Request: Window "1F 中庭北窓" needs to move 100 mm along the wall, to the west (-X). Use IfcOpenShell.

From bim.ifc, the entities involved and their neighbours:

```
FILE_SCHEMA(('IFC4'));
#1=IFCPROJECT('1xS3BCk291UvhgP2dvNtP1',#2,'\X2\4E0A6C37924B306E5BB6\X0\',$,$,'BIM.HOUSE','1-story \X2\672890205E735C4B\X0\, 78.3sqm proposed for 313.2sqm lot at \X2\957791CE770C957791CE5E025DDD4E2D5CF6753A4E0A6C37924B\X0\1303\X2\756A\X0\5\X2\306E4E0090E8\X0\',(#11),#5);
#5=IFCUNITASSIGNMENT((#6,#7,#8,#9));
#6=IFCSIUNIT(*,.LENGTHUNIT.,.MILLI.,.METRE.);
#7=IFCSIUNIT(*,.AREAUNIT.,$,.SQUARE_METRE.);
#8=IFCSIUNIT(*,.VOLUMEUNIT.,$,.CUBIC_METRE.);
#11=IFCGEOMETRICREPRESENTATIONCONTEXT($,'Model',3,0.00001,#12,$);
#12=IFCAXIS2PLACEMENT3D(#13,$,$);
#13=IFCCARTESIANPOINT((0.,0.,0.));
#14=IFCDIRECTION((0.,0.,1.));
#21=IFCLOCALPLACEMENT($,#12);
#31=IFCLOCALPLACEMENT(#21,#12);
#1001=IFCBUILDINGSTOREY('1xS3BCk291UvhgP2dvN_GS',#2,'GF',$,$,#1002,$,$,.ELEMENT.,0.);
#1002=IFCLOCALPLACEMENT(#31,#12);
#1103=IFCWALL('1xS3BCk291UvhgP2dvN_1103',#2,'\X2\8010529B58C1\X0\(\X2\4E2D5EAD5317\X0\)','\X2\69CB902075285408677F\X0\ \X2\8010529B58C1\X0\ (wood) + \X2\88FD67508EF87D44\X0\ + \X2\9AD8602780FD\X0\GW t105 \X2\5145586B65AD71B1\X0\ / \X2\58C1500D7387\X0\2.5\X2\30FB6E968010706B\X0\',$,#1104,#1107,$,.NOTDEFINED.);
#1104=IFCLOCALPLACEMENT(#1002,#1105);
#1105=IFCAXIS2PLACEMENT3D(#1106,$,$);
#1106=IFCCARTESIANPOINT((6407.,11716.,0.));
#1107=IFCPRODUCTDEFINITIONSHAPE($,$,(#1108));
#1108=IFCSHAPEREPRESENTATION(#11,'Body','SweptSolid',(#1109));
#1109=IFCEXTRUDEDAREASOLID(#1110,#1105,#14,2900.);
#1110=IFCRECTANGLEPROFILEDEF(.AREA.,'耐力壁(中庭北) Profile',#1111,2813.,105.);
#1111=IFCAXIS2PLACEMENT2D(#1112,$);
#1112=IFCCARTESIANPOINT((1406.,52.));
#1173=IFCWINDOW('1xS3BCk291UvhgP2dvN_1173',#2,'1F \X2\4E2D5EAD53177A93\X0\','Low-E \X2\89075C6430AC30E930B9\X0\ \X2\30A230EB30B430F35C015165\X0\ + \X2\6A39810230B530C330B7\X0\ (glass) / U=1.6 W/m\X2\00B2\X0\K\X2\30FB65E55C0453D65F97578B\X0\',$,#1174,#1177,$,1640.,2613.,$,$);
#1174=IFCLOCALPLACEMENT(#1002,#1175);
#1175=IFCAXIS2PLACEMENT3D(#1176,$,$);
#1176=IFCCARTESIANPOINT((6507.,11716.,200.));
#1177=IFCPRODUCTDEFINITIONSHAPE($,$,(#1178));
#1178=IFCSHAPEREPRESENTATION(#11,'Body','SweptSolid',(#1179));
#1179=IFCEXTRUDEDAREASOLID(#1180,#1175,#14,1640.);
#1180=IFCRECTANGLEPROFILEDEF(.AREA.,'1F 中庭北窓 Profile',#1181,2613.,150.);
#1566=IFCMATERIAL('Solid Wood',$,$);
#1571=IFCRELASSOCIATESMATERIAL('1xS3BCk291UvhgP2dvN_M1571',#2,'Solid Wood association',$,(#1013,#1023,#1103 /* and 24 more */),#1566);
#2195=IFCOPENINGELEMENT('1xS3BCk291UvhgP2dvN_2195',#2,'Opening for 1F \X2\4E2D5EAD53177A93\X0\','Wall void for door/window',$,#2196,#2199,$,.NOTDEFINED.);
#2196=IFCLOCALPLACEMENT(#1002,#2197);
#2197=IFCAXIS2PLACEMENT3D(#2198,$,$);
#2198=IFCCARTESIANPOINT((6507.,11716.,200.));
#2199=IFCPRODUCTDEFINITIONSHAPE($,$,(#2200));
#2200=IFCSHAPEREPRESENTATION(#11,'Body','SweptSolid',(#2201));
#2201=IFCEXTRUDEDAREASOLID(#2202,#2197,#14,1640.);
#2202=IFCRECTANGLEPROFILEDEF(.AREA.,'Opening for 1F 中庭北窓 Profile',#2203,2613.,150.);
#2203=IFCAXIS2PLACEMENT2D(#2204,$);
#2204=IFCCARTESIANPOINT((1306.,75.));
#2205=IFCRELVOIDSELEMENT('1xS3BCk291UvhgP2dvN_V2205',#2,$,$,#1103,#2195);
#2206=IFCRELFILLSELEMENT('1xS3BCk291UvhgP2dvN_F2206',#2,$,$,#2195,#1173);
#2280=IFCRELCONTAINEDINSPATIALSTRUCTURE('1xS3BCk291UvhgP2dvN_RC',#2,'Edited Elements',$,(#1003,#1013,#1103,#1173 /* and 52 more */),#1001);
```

```python
import ifcopenshell
import ifcopenshell.api.geometry
import ifcopenshell.util.placement

model = ifcopenshell.open("bim.ifc")

window = model.by_id(1173)
opening = window.FillsVoids[0].RelatingOpeningElement
wall = opening.VoidsElements[0].RelatingBuildingElement

wall_matrix = ifcopenshell.util.placement.get_local_placement(wall.ObjectPlacement)
shift = wall_matrix[:3, 0] * -100.0
before = ifcopenshell.util.placement.get_local_placement(window.ObjectPlacement)[:3, 3].copy()

# The window is not placed relative to its opening, so move both.
for product in (opening, window):
    matrix = ifcopenshell.util.placement.get_local_placement(product.ObjectPlacement)
    matrix[:3, 3] += shift
    ifcopenshell.api.geometry.edit_object_placement(model, product=product, matrix=matrix, is_si=False)

after = ifcopenshell.util.placement.get_local_placement(window.ObjectPlacement)[:3, 3]
print("window moved by", (after - before).round(3) + 0.0)

model.write("bim_rev.ifc")
```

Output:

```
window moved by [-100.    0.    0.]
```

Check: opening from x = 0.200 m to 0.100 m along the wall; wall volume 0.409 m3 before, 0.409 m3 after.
